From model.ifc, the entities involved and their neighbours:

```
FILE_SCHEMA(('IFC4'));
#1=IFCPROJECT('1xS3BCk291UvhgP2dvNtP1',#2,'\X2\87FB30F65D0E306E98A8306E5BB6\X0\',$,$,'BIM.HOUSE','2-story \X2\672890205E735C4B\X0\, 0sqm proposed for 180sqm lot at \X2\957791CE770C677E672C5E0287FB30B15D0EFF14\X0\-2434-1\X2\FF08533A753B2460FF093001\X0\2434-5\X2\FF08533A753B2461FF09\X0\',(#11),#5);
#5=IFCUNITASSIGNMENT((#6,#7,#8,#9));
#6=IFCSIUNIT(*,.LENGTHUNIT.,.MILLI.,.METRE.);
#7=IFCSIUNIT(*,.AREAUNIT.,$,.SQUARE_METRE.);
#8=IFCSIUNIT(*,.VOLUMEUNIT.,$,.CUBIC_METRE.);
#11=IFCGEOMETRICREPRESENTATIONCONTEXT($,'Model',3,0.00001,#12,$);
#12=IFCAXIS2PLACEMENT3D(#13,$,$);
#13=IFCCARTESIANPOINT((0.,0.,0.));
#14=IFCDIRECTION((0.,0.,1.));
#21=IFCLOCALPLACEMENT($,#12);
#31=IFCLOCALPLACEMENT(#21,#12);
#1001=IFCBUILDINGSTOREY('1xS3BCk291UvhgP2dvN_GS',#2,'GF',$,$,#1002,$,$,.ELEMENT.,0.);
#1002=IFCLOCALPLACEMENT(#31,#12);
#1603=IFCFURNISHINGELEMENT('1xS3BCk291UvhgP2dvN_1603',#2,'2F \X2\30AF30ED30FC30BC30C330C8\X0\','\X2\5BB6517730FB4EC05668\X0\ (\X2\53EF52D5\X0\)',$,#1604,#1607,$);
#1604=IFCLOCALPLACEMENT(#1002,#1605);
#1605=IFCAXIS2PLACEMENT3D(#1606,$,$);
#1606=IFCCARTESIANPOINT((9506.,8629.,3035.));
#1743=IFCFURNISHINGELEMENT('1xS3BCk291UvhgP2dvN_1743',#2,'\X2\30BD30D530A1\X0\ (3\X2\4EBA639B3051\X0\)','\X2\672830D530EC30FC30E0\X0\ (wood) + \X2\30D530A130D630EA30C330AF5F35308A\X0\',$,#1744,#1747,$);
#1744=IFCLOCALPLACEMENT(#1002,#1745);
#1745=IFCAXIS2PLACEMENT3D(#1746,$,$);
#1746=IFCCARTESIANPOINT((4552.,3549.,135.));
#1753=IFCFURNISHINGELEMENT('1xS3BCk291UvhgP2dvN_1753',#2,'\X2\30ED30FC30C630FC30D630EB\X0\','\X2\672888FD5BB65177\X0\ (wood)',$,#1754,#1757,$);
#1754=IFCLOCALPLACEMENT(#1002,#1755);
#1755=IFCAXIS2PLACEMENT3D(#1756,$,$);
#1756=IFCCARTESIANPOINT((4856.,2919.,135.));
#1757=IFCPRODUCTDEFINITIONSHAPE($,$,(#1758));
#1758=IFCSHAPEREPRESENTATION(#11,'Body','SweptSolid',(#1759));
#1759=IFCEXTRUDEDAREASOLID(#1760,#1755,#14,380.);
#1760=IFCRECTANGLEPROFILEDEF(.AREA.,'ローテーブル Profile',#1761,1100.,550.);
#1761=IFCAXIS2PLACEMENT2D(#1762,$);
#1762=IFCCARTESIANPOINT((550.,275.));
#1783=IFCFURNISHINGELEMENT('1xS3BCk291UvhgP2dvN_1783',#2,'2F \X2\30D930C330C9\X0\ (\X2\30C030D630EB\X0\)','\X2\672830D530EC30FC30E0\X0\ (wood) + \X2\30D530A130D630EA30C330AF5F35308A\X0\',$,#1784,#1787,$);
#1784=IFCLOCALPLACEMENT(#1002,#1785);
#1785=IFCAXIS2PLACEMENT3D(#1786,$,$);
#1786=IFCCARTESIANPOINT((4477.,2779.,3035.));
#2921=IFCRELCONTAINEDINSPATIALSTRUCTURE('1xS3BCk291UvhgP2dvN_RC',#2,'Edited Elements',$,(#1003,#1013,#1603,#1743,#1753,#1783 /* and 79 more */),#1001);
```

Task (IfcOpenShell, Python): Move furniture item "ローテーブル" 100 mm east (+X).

```python
import ifcopenshell
import ifcopenshell.api.geometry
import ifcopenshell.util.placement
import ifcopenshell.util.unit

model = ifcopenshell.open("model.ifc")
unit_scale = ifcopenshell.util.unit.calculate_unit_scale(model)

item = model.by_guid("1xS3BCk291UvhgP2dvN_1753")
matrix = ifcopenshell.util.placement.get_local_placement(item.ObjectPlacement)
matrix[0, 3] += 0.1 / unit_scale
ifcopenshell.api.geometry.edit_object_placement(model, product=item, matrix=matrix, is_si=False)

print(ifcopenshell.util.placement.get_local_placement(item.ObjectPlacement).round(3) + 0.0)

model.write("model-out.ifc")
```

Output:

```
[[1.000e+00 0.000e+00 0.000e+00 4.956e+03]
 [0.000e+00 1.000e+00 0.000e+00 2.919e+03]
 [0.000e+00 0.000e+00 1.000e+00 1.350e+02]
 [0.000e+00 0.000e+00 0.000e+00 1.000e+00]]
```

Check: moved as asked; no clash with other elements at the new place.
